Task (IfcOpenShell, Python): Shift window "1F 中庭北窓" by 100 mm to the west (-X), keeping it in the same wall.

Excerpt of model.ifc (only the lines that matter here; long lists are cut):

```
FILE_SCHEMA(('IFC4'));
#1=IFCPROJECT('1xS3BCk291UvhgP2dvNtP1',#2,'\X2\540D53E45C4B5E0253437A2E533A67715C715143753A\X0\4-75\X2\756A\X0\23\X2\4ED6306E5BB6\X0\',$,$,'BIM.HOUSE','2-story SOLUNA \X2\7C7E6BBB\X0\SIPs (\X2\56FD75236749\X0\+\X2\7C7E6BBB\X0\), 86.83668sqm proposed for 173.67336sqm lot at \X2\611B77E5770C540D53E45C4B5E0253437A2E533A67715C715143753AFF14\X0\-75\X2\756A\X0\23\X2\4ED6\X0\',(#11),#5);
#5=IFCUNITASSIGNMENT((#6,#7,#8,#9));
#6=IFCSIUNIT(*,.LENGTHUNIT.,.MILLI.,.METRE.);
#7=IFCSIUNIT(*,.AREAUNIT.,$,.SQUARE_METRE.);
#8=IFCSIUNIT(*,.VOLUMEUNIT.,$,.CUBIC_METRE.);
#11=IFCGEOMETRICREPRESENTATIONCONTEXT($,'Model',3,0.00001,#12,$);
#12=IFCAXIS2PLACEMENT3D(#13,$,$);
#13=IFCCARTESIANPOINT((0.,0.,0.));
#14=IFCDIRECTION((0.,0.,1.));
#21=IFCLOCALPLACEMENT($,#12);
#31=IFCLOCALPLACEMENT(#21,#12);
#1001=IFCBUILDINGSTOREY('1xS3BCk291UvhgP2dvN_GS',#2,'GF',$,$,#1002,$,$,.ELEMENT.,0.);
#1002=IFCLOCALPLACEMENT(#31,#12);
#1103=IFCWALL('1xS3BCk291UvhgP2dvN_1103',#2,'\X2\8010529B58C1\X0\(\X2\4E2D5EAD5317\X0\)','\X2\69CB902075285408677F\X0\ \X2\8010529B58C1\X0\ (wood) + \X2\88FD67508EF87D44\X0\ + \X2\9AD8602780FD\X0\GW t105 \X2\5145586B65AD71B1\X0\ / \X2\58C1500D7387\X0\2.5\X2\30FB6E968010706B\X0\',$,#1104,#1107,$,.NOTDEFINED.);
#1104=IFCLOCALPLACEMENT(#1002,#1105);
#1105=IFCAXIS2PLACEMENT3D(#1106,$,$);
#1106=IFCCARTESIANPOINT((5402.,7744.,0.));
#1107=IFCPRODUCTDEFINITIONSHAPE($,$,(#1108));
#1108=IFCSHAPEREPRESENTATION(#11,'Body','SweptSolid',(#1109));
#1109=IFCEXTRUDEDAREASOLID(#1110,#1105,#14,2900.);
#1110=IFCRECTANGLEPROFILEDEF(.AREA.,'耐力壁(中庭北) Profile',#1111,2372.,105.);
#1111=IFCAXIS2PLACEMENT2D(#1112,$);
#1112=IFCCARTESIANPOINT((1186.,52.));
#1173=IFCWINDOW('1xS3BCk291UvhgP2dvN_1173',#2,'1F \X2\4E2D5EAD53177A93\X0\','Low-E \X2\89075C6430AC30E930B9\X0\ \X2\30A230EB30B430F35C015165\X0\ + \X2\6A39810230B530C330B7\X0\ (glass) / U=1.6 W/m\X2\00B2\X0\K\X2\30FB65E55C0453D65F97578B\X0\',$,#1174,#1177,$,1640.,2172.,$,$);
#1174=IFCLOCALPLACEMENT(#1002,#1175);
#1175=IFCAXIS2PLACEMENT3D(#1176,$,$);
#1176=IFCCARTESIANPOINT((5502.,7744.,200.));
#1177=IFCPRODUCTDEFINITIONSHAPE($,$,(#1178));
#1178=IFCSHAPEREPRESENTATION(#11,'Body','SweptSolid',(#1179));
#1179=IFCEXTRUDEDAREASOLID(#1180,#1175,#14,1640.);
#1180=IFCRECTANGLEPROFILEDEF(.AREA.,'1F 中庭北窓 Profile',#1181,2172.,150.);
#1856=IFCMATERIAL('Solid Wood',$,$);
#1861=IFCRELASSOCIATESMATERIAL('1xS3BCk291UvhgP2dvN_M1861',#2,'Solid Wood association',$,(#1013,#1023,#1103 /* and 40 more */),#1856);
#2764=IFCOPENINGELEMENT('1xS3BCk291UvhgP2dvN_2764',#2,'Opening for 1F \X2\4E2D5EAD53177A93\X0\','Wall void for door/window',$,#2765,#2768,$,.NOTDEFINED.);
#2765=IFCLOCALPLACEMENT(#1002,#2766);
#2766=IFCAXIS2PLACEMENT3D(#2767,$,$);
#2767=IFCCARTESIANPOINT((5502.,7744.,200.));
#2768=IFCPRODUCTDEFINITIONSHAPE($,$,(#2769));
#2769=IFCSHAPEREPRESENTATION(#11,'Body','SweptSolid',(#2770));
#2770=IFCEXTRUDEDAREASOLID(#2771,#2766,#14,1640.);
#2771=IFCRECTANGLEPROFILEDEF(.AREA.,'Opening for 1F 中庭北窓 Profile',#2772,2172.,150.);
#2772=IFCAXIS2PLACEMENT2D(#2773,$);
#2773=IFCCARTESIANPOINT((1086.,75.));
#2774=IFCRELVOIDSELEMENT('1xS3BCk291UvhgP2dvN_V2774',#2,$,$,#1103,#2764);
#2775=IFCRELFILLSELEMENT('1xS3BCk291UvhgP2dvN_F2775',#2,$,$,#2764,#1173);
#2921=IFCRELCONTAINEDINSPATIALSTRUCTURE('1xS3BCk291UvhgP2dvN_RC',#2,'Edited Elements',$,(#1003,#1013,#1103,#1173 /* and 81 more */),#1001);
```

```python
import ifcopenshell
import ifcopenshell.api.geometry
import ifcopenshell.util.placement

model = ifcopenshell.open("model.ifc")

window = model.by_id(1173)
opening = window.FillsVoids[0].RelatingOpeningElement
wall = opening.VoidsElements[0].RelatingBuildingElement

wall_matrix = ifcopenshell.util.placement.get_local_placement(wall.ObjectPlacement)
shift = wall_matrix[:3, 0] * -100.0
before = ifcopenshell.util.placement.get_local_placement(window.ObjectPlacement)[:3, 3].copy()

# The window is not placed relative to its opening, so move both.
for product in (opening, window):
    matrix = ifcopenshell.util.placement.get_local_placement(product.ObjectPlacement)
    matrix[:3, 3] += shift
    ifcopenshell.api.geometry.edit_object_placement(model, product=product, matrix=matrix, is_si=False)

after = ifcopenshell.util.placement.get_local_placement(window.ObjectPlacement)[:3, 3]
print("window moved by", (after - before).round(3) + 0.0)

model.write("model_updated.ifc")
```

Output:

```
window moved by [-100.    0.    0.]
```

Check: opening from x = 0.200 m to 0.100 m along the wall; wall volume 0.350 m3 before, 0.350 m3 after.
